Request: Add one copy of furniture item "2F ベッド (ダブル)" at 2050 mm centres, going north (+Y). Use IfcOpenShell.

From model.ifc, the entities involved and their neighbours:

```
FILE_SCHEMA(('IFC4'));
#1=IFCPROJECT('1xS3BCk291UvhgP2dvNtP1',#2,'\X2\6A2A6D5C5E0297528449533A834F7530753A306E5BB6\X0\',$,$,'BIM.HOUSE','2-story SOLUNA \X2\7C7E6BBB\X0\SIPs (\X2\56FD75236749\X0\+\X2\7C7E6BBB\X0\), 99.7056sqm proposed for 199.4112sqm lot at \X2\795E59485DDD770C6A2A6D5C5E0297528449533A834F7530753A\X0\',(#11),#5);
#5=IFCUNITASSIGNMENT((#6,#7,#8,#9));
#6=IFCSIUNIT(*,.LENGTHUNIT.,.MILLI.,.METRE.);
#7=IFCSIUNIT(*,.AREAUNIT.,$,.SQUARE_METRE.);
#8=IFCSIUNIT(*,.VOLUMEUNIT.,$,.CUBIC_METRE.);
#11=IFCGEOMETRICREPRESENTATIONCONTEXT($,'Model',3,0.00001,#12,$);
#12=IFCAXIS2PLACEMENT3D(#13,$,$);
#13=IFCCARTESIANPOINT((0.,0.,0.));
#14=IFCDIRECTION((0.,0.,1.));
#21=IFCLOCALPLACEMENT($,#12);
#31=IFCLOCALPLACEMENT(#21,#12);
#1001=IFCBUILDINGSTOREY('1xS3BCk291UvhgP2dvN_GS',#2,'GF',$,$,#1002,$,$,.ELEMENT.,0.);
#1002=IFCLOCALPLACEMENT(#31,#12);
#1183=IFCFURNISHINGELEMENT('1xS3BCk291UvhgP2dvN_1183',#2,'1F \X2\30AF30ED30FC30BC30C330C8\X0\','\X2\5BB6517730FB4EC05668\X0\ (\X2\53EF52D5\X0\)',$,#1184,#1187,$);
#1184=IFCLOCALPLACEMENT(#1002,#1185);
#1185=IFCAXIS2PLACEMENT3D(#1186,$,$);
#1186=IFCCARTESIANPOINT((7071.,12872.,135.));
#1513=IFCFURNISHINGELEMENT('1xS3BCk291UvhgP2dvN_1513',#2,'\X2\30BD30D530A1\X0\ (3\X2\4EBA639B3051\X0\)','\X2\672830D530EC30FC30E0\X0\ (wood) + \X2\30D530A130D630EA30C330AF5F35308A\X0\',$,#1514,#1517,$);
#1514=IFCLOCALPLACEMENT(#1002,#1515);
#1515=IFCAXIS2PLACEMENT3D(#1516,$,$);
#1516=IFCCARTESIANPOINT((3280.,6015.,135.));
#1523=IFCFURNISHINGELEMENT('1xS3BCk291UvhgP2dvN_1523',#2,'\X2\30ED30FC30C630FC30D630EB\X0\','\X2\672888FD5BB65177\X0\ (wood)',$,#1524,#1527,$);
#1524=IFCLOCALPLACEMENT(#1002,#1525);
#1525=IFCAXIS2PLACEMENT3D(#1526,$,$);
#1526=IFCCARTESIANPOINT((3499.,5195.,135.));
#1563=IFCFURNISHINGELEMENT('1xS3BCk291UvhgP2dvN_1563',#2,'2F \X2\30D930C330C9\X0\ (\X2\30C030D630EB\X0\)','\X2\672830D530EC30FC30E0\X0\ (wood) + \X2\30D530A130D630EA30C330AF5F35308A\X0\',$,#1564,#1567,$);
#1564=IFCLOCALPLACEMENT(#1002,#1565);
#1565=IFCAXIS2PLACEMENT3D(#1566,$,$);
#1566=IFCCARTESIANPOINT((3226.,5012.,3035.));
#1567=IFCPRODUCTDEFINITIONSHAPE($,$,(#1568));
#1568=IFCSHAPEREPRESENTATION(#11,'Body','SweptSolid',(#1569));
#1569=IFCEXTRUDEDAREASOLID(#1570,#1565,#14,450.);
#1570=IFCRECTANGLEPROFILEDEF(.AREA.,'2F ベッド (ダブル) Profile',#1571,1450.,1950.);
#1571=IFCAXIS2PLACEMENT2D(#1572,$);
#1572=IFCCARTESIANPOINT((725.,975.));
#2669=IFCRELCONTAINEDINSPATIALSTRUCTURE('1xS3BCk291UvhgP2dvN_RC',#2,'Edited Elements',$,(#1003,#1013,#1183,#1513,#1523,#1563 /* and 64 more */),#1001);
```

```python
import numpy as np
import ifcopenshell
import ifcopenshell.api.geometry
import ifcopenshell.api.root
import ifcopenshell.util.element
import ifcopenshell.util.placement

model = ifcopenshell.open("model.ifc")


def reuse_history(source, copy):
    """copy_class also copies each property set's owner history, people and application; keep the originals."""
    for rel in copy.IsDefinedBy:
        if rel.is_a("IfcRelDefinesByProperties") and (history := rel.RelatingPropertyDefinition.OwnerHistory):
            rel.RelatingPropertyDefinition.OwnerHistory = source.OwnerHistory
            ifcopenshell.util.element.remove_deep2(model, history)


source = model.by_guid("1xS3BCk291UvhgP2dvN_1563")
base = ifcopenshell.util.placement.get_local_placement(source.ObjectPlacement)
step = np.array([0.0, 1.0, 0.0]) * 2050.0

for i in range(1, 2):
    copy = ifcopenshell.api.root.copy_class(model, product=source)
    copy.Representation = ifcopenshell.util.element.copy_deep(
        model, source.Representation, exclude=["IfcGeometricRepresentationContext", "IfcRepresentationMap"]
    )
    reuse_history(source, copy)
    matrix = base.copy()
    matrix[:3, 3] += i * step
    print("added at", matrix[:3, 3].round(3) + 0.0)
    ifcopenshell.api.geometry.edit_object_placement(model, product=copy, matrix=matrix, is_si=False)

model.write("model_rev.ifc")
```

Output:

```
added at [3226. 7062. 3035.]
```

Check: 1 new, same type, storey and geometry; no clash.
